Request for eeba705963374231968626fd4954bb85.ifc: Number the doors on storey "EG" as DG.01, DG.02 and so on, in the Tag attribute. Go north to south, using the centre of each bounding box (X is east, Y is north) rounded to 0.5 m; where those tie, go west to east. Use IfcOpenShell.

First a look at what the model holds.

```python
import ifcopenshell
import ifcopenshell.util.element
import ifcopenshell.util.placement

model = ifcopenshell.open("eeba705963374231968626fd4954bb85.ifc")
print(model.schema)
storey = next(s for s in model.by_type("IfcBuildingStorey") if s.Name == "EG")
doors = [e for e in ifcopenshell.util.element.get_decomposition(storey) if e.is_a("IfcDoor")]
for e in sorted(doors, key=lambda e: e.id()):
    origin = ifcopenshell.util.placement.get_local_placement(e.ObjectPlacement)[:3, 3]
    print(e.id(), e.Tag, e.Name, origin.round(2) + 0.0, sep=" | ")
```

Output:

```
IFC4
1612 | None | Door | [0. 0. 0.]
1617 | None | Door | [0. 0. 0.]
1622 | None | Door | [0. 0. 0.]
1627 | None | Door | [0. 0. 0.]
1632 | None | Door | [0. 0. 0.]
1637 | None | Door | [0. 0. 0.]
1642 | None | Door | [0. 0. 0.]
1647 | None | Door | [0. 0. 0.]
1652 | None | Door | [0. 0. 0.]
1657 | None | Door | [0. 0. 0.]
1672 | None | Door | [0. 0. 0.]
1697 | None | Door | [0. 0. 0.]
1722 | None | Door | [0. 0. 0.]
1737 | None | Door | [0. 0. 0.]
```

```python
import ifcopenshell
import ifcopenshell.geom
import ifcopenshell.util.element
import ifcopenshell.util.shape

model = ifcopenshell.open("eeba705963374231968626fd4954bb85.ifc")
settings = ifcopenshell.geom.settings()
settings.set("use-world-coords", True)


def centre(element):
    shape = ifcopenshell.geom.create_shape(settings, element)
    return ifcopenshell.util.shape.get_bbox_centroid(shape.geometry)


storey = next(s for s in model.by_type("IfcBuildingStorey") if s.Name == "EG")
doors = [e for e in ifcopenshell.util.element.get_decomposition(storey) if e.is_a("IfcDoor")]

# Insertion points can sit at a corner or the storey origin, so sort by the geometry (in metres).
centres = {e: centre(e) for e in doors}
doors.sort(key=lambda e: (-round(centres[e][1] / 0.5), centres[e][0]))

for i, e in enumerate(doors, start=1):
    number = f"DG.{i:02d}"
    e.Tag = number
    print(e.id(), number)

model.write("eeba705963374231968626fd4954bb85_updated.ifc")
```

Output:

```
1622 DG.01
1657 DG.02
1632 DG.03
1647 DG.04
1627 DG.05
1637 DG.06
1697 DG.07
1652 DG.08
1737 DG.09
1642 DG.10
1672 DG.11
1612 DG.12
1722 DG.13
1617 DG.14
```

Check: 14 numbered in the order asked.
